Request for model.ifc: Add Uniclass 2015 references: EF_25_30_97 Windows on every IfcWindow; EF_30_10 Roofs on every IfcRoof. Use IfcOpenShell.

First a look at what the model holds.

```python
import ifcopenshell

model = ifcopenshell.open("model.ifc")
print(model.schema)
print("classifications:", [c.Name for c in model.by_type("IfcClassification")])
for ifc_class in ("IfcDoor", "IfcRoof", "IfcStair", "IfcWall", "IfcWindow"):
    print(ifc_class, len(model.by_type(ifc_class)))
```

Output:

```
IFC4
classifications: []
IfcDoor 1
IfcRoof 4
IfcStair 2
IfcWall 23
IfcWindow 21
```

```python
import ifcopenshell
import ifcopenshell.api.classification

model = ifcopenshell.open("model.ifc")

system = ifcopenshell.api.classification.add_classification(model, classification="Uniclass 2015")

codes = {
    "IfcWindow": ("EF_25_30_97", "Windows"),
    "IfcRoof": ("EF_30_10", "Roofs"),
}
for ifc_class, (code, name) in codes.items():
    products = model.by_type(ifc_class)
    ifcopenshell.api.classification.add_reference(
        model, products=products, classification=system, identification=code, name=name
    )
    print(code, len(products))

model.write("model_edited.ifc")
```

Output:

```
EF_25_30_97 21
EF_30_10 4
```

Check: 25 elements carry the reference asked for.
